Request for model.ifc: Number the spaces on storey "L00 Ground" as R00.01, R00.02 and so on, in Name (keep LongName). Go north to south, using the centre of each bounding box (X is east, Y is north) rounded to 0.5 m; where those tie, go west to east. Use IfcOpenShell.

First a look at what the model holds.

```python
import ifcopenshell
import ifcopenshell.util.element
import ifcopenshell.util.placement

model = ifcopenshell.open("model.ifc")
print(model.schema)
storey = next(s for s in model.by_type("IfcBuildingStorey") if s.Name == "L00 Ground")
spaces = [e for e in ifcopenshell.util.element.get_decomposition(storey) if e.is_a("IfcSpace")]
for e in sorted(spaces, key=lambda e: e.id()):
    origin = ifcopenshell.util.placement.get_local_placement(e.ObjectPlacement)[:3, 3]
    print(e.id(), e.Name, e.LongName, origin.round(2) + 0.0, sep=" | ")
```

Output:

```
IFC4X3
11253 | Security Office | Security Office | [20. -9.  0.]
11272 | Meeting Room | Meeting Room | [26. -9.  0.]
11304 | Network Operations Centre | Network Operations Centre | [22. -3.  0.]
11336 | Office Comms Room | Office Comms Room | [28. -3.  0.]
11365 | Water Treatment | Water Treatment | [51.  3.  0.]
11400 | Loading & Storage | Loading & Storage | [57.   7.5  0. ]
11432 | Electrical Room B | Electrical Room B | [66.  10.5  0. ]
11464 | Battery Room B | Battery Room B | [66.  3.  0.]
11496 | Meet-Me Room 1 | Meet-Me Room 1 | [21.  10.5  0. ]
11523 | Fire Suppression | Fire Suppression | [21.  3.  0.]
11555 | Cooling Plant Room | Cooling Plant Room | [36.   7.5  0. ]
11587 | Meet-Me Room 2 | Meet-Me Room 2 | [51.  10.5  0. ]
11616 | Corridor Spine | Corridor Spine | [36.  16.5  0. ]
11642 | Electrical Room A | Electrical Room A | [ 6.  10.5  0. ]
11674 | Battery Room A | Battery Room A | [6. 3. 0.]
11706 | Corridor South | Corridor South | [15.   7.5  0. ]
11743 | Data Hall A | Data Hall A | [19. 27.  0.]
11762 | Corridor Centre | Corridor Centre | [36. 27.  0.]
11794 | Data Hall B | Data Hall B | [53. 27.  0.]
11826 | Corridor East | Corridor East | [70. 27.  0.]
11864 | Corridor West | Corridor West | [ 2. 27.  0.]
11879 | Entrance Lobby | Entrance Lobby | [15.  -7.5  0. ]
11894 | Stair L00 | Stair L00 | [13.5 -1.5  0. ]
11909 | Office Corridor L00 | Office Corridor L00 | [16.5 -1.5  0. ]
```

```python
import ifcopenshell
import ifcopenshell.geom
import ifcopenshell.util.element
import ifcopenshell.util.shape

model = ifcopenshell.open("model.ifc")
settings = ifcopenshell.geom.settings()
settings.set("use-world-coords", True)


def centre(element):
    shape = ifcopenshell.geom.create_shape(settings, element)
    return ifcopenshell.util.shape.get_bbox_centroid(shape.geometry)


storey = next(s for s in model.by_type("IfcBuildingStorey") if s.Name == "L00 Ground")
spaces = [e for e in ifcopenshell.util.element.get_decomposition(storey) if e.is_a("IfcSpace")]

# Insertion points can sit at a corner or the storey origin, so sort by the geometry (in metres).
centres = {e: centre(e) for e in spaces}
spaces.sort(key=lambda e: (-round(centres[e][1] / 0.5), centres[e][0]))

for i, e in enumerate(spaces, start=1):
    number = f"R00.{i:02d}"
    e.Name = number
    print(e.id(), number)

model.write("model_v2.ifc")
```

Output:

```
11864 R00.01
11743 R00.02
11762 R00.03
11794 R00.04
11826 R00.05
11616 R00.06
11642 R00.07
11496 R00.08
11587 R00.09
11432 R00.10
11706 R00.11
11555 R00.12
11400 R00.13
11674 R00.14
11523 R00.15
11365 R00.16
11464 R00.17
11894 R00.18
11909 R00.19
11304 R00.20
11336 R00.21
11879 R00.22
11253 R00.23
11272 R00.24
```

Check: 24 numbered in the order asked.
